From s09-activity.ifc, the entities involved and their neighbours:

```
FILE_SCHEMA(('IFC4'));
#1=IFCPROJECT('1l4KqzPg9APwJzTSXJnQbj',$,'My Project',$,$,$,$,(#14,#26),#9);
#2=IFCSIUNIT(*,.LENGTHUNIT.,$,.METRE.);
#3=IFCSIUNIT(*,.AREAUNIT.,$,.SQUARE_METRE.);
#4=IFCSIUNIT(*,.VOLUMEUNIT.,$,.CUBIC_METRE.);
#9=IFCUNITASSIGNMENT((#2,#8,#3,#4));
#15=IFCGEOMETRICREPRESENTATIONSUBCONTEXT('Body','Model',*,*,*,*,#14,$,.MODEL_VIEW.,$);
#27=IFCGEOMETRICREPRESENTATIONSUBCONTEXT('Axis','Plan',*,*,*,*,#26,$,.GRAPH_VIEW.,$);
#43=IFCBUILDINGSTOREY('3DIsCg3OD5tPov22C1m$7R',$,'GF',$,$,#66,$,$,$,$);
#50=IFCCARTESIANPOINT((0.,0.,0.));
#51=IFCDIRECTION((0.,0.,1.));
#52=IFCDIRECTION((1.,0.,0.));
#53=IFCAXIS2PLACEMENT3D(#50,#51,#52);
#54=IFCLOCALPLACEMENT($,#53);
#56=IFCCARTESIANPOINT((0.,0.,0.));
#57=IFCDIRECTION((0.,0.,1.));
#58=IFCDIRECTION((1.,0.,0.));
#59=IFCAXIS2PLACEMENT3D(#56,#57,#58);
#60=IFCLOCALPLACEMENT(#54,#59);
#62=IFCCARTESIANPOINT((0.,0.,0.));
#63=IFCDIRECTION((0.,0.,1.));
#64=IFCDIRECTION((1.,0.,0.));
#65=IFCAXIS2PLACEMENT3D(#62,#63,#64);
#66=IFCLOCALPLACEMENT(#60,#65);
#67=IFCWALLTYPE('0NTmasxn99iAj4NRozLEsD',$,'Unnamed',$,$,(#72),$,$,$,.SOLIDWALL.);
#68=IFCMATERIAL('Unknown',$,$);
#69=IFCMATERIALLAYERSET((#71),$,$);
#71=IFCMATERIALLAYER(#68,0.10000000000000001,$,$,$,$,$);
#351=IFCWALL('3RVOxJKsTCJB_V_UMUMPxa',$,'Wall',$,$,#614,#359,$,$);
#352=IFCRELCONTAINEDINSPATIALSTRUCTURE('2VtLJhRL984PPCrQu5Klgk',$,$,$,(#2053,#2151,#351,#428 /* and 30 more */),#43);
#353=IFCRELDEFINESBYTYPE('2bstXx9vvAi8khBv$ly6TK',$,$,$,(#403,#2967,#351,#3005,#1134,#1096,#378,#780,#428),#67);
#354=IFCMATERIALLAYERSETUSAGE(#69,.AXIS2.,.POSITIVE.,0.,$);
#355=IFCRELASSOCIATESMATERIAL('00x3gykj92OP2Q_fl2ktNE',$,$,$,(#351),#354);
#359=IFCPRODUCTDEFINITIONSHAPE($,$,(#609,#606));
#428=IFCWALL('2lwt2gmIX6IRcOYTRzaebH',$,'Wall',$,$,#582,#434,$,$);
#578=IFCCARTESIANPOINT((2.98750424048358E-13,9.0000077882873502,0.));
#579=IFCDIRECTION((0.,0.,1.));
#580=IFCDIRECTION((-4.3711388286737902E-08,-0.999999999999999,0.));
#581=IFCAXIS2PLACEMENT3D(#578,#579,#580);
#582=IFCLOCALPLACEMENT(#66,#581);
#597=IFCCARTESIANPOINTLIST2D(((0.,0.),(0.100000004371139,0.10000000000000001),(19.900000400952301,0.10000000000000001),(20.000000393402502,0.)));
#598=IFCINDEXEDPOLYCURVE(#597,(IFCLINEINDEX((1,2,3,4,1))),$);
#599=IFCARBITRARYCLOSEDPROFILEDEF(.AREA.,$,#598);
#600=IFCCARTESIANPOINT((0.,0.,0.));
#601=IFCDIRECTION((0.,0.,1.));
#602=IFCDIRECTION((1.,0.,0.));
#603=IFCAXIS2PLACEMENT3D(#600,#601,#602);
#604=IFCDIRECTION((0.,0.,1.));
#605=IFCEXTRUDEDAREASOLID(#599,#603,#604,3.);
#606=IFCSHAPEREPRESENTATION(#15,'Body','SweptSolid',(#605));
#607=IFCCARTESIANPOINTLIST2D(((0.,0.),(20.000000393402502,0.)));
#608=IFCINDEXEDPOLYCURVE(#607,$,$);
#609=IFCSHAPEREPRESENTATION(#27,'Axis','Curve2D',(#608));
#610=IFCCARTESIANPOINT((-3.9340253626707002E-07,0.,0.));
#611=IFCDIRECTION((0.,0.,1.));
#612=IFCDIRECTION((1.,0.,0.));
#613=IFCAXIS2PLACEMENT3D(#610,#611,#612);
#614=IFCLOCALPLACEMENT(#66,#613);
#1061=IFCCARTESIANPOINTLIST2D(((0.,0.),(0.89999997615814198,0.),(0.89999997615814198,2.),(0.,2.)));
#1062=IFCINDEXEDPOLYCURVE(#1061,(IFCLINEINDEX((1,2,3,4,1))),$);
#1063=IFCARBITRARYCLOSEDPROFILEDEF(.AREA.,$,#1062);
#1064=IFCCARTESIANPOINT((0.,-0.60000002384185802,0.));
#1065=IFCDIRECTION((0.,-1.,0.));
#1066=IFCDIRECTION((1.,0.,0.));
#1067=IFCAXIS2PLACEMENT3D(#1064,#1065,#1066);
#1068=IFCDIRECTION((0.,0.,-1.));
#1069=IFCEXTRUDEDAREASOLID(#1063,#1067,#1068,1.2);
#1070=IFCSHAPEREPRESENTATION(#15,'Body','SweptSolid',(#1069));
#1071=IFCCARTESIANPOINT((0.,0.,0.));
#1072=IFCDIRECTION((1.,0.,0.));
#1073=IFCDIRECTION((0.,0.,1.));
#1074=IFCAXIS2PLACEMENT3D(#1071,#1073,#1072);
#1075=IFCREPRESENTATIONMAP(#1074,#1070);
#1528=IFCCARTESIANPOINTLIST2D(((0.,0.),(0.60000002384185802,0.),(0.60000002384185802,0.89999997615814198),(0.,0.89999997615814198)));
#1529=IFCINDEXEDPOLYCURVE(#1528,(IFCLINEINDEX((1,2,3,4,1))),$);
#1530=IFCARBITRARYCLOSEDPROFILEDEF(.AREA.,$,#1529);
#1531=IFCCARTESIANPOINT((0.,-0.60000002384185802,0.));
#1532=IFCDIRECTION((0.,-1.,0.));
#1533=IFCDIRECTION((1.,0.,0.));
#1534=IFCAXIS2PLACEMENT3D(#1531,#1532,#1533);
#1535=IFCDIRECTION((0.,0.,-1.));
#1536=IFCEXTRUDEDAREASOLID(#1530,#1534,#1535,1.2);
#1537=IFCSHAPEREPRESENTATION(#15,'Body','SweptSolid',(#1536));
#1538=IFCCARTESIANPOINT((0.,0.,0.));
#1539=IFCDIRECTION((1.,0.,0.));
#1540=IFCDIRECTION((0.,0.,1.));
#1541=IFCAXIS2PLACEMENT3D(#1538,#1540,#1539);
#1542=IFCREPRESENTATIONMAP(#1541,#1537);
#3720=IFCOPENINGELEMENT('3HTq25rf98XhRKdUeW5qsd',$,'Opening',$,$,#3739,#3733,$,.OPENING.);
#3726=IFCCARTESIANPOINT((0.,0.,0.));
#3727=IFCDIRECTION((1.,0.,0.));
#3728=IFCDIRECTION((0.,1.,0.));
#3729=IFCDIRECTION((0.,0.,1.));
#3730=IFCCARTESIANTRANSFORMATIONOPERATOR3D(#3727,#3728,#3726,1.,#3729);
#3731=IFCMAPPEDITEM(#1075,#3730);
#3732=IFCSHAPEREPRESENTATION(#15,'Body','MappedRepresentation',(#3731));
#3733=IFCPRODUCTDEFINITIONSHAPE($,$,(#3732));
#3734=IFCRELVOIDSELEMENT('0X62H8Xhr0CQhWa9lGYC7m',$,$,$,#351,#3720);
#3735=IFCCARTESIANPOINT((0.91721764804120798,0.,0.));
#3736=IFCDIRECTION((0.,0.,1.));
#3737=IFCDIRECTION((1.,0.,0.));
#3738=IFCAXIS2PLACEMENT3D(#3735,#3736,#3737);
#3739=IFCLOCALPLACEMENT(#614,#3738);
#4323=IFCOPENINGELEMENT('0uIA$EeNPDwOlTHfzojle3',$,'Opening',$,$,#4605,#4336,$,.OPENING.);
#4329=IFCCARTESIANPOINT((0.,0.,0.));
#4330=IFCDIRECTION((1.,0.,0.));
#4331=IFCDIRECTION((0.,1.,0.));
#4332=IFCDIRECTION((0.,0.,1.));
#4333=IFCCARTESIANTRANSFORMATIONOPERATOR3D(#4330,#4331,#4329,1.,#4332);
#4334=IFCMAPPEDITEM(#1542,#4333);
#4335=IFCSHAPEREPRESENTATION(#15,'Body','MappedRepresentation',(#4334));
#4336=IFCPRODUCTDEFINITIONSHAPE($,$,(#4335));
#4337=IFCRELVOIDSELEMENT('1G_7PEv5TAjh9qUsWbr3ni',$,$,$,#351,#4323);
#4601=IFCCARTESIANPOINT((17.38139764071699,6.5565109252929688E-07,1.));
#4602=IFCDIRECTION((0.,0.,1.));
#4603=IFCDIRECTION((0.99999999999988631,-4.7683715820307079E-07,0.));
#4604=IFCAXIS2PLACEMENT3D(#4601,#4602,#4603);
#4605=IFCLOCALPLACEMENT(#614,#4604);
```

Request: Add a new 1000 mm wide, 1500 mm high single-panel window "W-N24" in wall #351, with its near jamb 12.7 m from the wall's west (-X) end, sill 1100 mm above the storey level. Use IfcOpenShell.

```python
import numpy as np
import ifcopenshell
import ifcopenshell.api.feature
import ifcopenshell.api.geometry
import ifcopenshell.api.root
import ifcopenshell.api.spatial
import ifcopenshell.geom
import ifcopenshell.util.element
import ifcopenshell.util.placement
import ifcopenshell.util.representation
import ifcopenshell.util.shape
import ifcopenshell.util.unit

model = ifcopenshell.open("s09-activity.ifc")
unit_scale = ifcopenshell.util.unit.calculate_unit_scale(model)
settings = ifcopenshell.geom.settings()


def volume(element):
    """Net volume in cubic metres, openings subtracted."""
    shape = ifcopenshell.geom.create_shape(settings, element)
    return ifcopenshell.util.shape.get_volume(shape.geometry)


wall = model.by_id(351)
storey = ifcopenshell.util.element.get_container(wall, ifc_class="IfcBuildingStorey")
context = ifcopenshell.util.representation.get_context(model, "Model", "Body", "MODEL_VIEW")
before = volume(wall)

width, height, from_end, sill = 1, 1.5, 12.7, 1.1  # metres

# The wall runs along its own X axis, and the end named is its -X end.
wall_shape = ifcopenshell.geom.create_shape(settings, wall)
x, y, z = ifcopenshell.util.shape.get_vertices(wall_shape.geometry).T
start = x.min() + from_end
face, thickness = float(y.min()), float(y.max() - y.min())
wall_matrix = ifcopenshell.util.placement.get_local_placement(wall.ObjectPlacement)
level = ifcopenshell.util.placement.get_local_placement(storey.ObjectPlacement)[2, 3]


def in_wall(x, y):
    """Placement at x, y metres in the wall's axes, at sill height."""
    matrix = wall_matrix.copy()
    matrix[:, 3] = wall_matrix @ np.array([x / unit_scale, y / unit_scale, 0.0, 1.0])
    matrix[2, 3] = level + sill / unit_scale
    return matrix


# Opening: a box that overshoots both wall faces by 50 mm.
opening = ifcopenshell.api.root.create_entity(model, ifc_class="IfcOpeningElement", predefined_type="OPENING")
box = ifcopenshell.api.geometry.add_wall_representation(
    model, context=context, length=width, height=height, thickness=thickness + 0.1
)
ifcopenshell.api.geometry.assign_representation(model, product=opening, representation=box)
ifcopenshell.api.geometry.edit_object_placement(model, product=opening, matrix=in_wall(start, face - 0.05), is_si=False)
ifcopenshell.api.feature.add_feature(model, feature=opening, element=wall)

window = ifcopenshell.api.root.create_entity(model, ifc_class="IfcWindow", name="W-N24", predefined_type="WINDOW")
window.OverallWidth, window.OverallHeight = width / unit_scale, height / unit_scale
window.PartitioningType = "SINGLE_PANEL"
body = ifcopenshell.api.geometry.add_window_representation(
    model,
    context=context,
    overall_width=window.OverallWidth,
    overall_height=window.OverallHeight,
    partition_type="SINGLE_PANEL",
)
ifcopenshell.api.geometry.assign_representation(model, product=window, representation=body)
ifcopenshell.api.spatial.assign_container(model, products=[window], relating_structure=storey)
ifcopenshell.api.feature.add_filling(model, opening=opening, element=window)

# Centre the window in the wall's thickness.
ifcopenshell.api.geometry.edit_object_placement(model, product=window, matrix=in_wall(start, face), is_si=False)
window_shape = ifcopenshell.geom.create_shape(settings, window)
depth = ifcopenshell.util.shape.get_vertices(window_shape.geometry)[:, 1]
offset = face + thickness / 2 - (depth.min() + depth.max()) / 2
ifcopenshell.api.geometry.edit_object_placement(model, product=window, matrix=in_wall(start, offset), is_si=False)

after = volume(wall)

print(f"wall volume {before:.3f} -> {after:.3f} m3")

model.write("s09-activity_updated.ifc")
```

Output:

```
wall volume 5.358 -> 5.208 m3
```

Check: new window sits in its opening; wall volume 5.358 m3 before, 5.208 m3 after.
